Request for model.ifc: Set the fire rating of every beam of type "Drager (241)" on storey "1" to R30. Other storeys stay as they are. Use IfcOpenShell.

First a look at what the model holds.

```python
import ifcopenshell
import ifcopenshell.util.element

model = ifcopenshell.open("model.ifc")
print(model.schema)
storey = next(s for s in model.by_type("IfcBuildingStorey") if s.Name == "1")
beams = [e for e in ifcopenshell.util.element.get_decomposition(storey) if e.is_a("IfcBeam")]
seen = {}
for e in beams:
    element_type = ifcopenshell.util.element.get_type(e)
    key = (element_type.Name if element_type != e and element_type else None, ifcopenshell.util.element.get_pset(e, "Pset_BeamCommon", "FireRating"))
    seen[key] = seen.get(key, 0) + 1
for (name, value), count in sorted(seen.items(), key=str):
    print(count, "x", name, "|", value)
```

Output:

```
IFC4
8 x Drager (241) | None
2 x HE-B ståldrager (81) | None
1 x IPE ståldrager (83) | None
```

```python
import ifcopenshell
import ifcopenshell.api.pset
import ifcopenshell.util.element

model = ifcopenshell.open("model.ifc")

storey = next(s for s in model.by_type("IfcBuildingStorey") if s.Name == "1")
beams = [e for e in ifcopenshell.util.element.get_decomposition(storey) if e.is_a("IfcBeam")]

count = 0
for e in beams:
    element_type = ifcopenshell.util.element.get_type(e)
    if element_type in (None, e) or element_type.Name != "Drager (241)":
        continue
    # add_pset returns the element's existing set when there is one.
    pset = ifcopenshell.api.pset.add_pset(model, product=e, name="Pset_BeamCommon")
    ifcopenshell.api.pset.edit_pset(model, pset=pset, properties={"FireRating": "R30"})
    count += 1

print(count, "beams updated")

model.write("model-out.ifc")
```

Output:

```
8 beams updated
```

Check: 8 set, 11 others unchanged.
